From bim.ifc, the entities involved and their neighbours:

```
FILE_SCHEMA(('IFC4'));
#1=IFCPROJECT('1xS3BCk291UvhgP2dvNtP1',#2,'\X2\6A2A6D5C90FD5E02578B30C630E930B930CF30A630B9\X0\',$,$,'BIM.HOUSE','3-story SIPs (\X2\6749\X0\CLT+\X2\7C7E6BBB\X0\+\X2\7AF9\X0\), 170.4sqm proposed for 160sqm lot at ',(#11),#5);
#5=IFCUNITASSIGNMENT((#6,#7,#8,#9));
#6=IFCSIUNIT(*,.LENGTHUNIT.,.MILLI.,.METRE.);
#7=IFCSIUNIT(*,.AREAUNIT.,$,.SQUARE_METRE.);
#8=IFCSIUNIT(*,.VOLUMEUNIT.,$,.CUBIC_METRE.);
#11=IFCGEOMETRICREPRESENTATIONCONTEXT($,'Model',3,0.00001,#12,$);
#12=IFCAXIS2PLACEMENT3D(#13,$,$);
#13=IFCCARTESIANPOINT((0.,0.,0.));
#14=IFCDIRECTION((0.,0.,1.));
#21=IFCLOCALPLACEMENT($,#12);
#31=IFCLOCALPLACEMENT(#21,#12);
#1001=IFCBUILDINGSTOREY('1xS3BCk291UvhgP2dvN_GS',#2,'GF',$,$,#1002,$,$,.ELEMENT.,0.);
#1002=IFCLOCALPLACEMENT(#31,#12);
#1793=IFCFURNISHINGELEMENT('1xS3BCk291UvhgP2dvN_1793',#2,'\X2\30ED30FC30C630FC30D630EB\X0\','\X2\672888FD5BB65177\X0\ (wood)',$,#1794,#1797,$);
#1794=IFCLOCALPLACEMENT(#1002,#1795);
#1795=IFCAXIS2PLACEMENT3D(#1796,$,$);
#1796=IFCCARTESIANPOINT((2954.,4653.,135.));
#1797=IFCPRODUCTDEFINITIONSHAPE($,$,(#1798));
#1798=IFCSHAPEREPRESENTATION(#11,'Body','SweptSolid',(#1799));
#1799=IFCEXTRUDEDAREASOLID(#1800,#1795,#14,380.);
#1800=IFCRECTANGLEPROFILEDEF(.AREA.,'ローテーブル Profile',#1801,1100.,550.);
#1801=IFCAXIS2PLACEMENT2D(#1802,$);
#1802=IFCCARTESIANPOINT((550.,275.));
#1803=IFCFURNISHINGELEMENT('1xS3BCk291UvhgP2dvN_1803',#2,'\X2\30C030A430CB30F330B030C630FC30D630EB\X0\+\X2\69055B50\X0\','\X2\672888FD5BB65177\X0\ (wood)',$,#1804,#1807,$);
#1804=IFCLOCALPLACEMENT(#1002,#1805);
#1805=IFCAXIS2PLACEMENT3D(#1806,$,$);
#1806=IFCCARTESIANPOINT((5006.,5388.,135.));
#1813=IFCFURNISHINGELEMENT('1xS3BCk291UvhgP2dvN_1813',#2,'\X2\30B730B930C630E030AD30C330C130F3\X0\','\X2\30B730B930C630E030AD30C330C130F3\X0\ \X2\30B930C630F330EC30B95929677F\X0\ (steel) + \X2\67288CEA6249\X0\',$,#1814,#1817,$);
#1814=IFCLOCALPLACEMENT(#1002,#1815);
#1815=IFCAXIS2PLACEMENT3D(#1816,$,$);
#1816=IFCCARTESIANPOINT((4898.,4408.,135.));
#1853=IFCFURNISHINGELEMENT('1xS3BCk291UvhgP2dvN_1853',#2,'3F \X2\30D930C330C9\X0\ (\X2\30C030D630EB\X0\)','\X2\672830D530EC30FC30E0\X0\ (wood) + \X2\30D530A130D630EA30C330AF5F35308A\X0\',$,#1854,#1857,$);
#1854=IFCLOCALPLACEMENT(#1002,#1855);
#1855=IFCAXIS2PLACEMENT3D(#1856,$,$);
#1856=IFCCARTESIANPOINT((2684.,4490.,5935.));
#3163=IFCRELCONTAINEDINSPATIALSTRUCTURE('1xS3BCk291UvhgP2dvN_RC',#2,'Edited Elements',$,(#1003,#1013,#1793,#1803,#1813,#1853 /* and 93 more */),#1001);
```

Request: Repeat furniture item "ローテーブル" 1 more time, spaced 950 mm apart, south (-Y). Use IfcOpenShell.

```python
import numpy as np
import ifcopenshell
import ifcopenshell.api.geometry
import ifcopenshell.api.root
import ifcopenshell.util.element
import ifcopenshell.util.placement
import ifcopenshell.util.unit

model = ifcopenshell.open("bim.ifc")
unit_scale = ifcopenshell.util.unit.calculate_unit_scale(model)


def reuse_history(source, copy):
    """copy_class also copies each property set's owner history, people and application; keep the originals."""
    for rel in copy.IsDefinedBy:
        if rel.is_a("IfcRelDefinesByProperties") and (history := rel.RelatingPropertyDefinition.OwnerHistory):
            rel.RelatingPropertyDefinition.OwnerHistory = source.OwnerHistory
            ifcopenshell.util.element.remove_deep2(model, history)


source = model.by_guid("1xS3BCk291UvhgP2dvN_1793")
base = ifcopenshell.util.placement.get_local_placement(source.ObjectPlacement)
step = np.array([0.0, -1.0, 0.0]) * 0.95 / unit_scale

for i in range(1, 2):
    copy = ifcopenshell.api.root.copy_class(model, product=source)
    copy.Representation = ifcopenshell.util.element.copy_deep(
        model, source.Representation, exclude=["IfcGeometricRepresentationContext", "IfcRepresentationMap"]
    )
    reuse_history(source, copy)
    matrix = base.copy()
    matrix[:3, 3] += i * step
    print("added at", matrix[:3, 3].round(3) + 0.0)
    ifcopenshell.api.geometry.edit_object_placement(model, product=copy, matrix=matrix, is_si=False)

model.write("bim_updated.ifc")
```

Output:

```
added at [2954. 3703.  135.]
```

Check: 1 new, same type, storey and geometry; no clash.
